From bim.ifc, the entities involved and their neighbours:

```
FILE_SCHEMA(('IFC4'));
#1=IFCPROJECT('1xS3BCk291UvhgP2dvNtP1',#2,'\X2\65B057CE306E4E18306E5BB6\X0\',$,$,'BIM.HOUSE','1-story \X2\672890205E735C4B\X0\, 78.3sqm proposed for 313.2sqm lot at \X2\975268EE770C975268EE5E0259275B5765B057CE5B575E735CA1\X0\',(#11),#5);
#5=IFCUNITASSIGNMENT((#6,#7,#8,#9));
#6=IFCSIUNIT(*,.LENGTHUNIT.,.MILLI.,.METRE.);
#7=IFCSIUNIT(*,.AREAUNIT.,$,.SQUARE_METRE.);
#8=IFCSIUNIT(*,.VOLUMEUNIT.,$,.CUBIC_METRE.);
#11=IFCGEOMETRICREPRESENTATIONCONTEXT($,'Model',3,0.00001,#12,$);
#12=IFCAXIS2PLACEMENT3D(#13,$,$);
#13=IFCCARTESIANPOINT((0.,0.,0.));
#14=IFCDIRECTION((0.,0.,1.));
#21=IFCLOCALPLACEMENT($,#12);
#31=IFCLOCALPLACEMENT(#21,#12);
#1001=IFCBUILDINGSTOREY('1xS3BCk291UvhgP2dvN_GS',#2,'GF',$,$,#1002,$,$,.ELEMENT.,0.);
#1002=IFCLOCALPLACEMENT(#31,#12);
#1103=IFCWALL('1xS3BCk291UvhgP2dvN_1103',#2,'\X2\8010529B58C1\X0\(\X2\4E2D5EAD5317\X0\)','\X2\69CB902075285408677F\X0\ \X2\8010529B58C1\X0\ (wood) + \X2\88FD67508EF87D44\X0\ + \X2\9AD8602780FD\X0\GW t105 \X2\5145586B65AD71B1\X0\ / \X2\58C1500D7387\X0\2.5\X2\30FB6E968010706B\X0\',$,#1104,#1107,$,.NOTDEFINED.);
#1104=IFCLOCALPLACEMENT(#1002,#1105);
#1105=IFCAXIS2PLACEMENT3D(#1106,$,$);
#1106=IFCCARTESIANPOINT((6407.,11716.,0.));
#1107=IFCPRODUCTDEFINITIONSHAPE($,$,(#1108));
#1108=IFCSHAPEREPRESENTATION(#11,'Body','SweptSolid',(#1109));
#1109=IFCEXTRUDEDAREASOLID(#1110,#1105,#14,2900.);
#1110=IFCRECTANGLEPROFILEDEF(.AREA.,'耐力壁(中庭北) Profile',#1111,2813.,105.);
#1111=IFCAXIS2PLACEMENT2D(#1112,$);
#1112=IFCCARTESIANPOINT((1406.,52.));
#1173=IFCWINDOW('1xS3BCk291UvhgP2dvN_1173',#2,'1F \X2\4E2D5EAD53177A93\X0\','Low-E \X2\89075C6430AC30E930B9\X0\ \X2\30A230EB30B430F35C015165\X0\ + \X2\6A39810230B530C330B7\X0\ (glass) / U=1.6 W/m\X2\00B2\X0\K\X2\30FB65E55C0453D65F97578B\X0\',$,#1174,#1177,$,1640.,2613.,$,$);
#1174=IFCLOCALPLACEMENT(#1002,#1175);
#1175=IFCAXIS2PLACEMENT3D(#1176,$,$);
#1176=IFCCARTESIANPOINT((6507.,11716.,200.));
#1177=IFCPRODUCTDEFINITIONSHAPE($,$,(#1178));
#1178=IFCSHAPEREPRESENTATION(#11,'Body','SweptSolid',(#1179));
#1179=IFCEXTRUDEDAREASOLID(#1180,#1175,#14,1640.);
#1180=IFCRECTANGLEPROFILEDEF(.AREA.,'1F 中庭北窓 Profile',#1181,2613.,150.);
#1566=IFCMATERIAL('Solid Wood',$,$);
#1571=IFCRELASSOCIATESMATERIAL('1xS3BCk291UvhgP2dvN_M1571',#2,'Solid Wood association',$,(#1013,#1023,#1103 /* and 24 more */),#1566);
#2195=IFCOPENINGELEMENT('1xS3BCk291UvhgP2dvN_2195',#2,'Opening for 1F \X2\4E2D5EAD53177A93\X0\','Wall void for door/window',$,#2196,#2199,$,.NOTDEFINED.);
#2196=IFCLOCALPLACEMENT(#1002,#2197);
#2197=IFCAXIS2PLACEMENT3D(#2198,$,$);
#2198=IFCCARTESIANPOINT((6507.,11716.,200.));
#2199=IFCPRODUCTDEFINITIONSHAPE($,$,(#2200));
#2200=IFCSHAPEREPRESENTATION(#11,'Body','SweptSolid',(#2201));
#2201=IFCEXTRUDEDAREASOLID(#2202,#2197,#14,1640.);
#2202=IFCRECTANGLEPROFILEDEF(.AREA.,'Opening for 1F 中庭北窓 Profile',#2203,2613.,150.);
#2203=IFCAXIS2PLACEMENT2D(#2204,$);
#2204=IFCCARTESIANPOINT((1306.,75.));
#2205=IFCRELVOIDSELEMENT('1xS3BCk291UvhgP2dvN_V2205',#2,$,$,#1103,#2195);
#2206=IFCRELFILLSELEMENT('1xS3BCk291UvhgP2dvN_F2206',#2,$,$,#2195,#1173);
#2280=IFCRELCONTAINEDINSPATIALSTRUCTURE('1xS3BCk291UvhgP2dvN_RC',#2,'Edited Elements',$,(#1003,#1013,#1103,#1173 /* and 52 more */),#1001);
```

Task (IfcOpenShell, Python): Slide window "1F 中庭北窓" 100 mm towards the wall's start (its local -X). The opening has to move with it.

```python
import ifcopenshell
import ifcopenshell.api.geometry
import ifcopenshell.util.placement
import ifcopenshell.util.unit

model = ifcopenshell.open("bim.ifc")
unit_scale = ifcopenshell.util.unit.calculate_unit_scale(model)

window = model.by_id(1173)
opening = window.FillsVoids[0].RelatingOpeningElement
wall = opening.VoidsElements[0].RelatingBuildingElement

wall_matrix = ifcopenshell.util.placement.get_local_placement(wall.ObjectPlacement)
shift = wall_matrix[:3, 0] * -0.1 / unit_scale
before = ifcopenshell.util.placement.get_local_placement(window.ObjectPlacement)[:3, 3].copy()

# The window is not placed relative to its opening, so move both.
for product in (opening, window):
    matrix = ifcopenshell.util.placement.get_local_placement(product.ObjectPlacement)
    matrix[:3, 3] += shift
    ifcopenshell.api.geometry.edit_object_placement(model, product=product, matrix=matrix, is_si=False)

after = ifcopenshell.util.placement.get_local_placement(window.ObjectPlacement)[:3, 3]
print("window moved by", (after - before).round(3) + 0.0)

model.write("bim_v2.ifc")
```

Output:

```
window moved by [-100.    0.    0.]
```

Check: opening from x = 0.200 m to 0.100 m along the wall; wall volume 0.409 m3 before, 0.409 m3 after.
